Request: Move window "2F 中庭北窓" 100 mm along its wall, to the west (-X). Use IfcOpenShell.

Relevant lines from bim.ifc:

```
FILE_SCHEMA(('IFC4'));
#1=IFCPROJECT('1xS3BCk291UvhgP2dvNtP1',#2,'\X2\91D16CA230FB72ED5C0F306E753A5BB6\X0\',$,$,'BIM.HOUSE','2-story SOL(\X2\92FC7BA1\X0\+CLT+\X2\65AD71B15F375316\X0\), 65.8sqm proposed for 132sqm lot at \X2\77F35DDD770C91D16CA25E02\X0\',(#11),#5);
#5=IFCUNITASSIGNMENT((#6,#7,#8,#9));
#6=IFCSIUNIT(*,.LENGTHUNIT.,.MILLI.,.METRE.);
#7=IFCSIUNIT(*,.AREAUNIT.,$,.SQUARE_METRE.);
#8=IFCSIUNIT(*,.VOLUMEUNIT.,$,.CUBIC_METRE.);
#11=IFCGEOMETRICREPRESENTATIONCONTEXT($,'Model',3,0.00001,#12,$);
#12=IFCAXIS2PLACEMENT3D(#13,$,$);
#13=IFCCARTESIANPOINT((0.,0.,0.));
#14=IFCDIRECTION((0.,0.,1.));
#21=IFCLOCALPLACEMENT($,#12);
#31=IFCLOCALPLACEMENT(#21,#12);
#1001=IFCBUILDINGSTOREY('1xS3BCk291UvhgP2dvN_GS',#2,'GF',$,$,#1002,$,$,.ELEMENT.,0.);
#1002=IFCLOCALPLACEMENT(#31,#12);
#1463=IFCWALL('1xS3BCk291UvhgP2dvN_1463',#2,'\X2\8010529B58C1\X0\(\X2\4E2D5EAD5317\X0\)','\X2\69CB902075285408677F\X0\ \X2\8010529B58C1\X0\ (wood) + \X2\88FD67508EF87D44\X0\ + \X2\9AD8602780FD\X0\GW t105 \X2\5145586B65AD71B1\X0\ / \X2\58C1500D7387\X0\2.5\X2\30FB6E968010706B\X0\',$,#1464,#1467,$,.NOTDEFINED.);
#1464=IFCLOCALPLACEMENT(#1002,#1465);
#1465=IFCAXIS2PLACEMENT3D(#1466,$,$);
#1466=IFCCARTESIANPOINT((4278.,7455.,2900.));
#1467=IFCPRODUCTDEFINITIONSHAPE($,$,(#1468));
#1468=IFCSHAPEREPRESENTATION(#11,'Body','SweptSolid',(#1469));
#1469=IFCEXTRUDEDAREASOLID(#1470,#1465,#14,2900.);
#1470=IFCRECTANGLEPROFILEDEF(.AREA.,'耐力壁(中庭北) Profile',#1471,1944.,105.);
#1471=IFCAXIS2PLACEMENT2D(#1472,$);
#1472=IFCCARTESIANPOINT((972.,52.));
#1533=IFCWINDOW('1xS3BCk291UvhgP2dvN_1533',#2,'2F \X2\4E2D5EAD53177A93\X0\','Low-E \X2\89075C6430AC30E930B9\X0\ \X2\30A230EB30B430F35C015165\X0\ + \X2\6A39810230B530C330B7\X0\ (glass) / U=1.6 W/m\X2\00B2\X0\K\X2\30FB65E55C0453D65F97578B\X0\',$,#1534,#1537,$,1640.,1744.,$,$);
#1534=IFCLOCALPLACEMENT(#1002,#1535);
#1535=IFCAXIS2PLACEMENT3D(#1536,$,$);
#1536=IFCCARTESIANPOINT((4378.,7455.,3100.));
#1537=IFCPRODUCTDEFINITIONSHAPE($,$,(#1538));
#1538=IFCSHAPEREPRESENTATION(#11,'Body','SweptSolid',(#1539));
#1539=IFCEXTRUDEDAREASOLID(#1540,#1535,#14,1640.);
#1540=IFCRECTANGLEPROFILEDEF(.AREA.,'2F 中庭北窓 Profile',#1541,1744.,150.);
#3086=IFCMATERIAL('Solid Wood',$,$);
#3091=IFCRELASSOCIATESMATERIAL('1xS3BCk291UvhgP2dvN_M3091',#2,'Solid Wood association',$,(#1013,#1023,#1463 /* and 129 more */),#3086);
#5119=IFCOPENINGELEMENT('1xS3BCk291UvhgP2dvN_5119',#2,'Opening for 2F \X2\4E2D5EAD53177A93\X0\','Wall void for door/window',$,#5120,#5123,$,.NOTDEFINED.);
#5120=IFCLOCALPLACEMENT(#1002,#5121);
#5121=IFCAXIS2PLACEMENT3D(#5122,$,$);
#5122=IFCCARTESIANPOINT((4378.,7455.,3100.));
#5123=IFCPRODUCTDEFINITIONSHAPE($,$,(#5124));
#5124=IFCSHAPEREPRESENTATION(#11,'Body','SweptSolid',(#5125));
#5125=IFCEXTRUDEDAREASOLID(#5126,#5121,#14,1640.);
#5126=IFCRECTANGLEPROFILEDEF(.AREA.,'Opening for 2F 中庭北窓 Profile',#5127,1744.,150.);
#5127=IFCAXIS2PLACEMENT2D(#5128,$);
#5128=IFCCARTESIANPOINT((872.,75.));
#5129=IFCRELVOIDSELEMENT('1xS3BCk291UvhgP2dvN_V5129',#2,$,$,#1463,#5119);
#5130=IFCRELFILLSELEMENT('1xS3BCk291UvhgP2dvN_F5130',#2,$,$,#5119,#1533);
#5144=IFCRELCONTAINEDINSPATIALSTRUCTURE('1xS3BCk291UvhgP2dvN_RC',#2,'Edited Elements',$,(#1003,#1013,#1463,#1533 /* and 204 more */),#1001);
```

```python
import ifcopenshell
import ifcopenshell.api.geometry
import ifcopenshell.util.placement
import ifcopenshell.util.unit

model = ifcopenshell.open("bim.ifc")
unit_scale = ifcopenshell.util.unit.calculate_unit_scale(model)

window = model.by_guid("1xS3BCk291UvhgP2dvN_1533")
opening = window.FillsVoids[0].RelatingOpeningElement
wall = opening.VoidsElements[0].RelatingBuildingElement

wall_matrix = ifcopenshell.util.placement.get_local_placement(wall.ObjectPlacement)
shift = wall_matrix[:3, 0] * -0.1 / unit_scale
before = ifcopenshell.util.placement.get_local_placement(window.ObjectPlacement)[:3, 3].copy()

# The window is not placed relative to its opening, so move both.
for product in (opening, window):
    matrix = ifcopenshell.util.placement.get_local_placement(product.ObjectPlacement)
    matrix[:3, 3] += shift
    ifcopenshell.api.geometry.edit_object_placement(model, product=product, matrix=matrix, is_si=False)

after = ifcopenshell.util.placement.get_local_placement(window.ObjectPlacement)[:3, 3]
print("window moved by", (after - before).round(3) + 0.0)

model.write("bim_updated.ifc")
```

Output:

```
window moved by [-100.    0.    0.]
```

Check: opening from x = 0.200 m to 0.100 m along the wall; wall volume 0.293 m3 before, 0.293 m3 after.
